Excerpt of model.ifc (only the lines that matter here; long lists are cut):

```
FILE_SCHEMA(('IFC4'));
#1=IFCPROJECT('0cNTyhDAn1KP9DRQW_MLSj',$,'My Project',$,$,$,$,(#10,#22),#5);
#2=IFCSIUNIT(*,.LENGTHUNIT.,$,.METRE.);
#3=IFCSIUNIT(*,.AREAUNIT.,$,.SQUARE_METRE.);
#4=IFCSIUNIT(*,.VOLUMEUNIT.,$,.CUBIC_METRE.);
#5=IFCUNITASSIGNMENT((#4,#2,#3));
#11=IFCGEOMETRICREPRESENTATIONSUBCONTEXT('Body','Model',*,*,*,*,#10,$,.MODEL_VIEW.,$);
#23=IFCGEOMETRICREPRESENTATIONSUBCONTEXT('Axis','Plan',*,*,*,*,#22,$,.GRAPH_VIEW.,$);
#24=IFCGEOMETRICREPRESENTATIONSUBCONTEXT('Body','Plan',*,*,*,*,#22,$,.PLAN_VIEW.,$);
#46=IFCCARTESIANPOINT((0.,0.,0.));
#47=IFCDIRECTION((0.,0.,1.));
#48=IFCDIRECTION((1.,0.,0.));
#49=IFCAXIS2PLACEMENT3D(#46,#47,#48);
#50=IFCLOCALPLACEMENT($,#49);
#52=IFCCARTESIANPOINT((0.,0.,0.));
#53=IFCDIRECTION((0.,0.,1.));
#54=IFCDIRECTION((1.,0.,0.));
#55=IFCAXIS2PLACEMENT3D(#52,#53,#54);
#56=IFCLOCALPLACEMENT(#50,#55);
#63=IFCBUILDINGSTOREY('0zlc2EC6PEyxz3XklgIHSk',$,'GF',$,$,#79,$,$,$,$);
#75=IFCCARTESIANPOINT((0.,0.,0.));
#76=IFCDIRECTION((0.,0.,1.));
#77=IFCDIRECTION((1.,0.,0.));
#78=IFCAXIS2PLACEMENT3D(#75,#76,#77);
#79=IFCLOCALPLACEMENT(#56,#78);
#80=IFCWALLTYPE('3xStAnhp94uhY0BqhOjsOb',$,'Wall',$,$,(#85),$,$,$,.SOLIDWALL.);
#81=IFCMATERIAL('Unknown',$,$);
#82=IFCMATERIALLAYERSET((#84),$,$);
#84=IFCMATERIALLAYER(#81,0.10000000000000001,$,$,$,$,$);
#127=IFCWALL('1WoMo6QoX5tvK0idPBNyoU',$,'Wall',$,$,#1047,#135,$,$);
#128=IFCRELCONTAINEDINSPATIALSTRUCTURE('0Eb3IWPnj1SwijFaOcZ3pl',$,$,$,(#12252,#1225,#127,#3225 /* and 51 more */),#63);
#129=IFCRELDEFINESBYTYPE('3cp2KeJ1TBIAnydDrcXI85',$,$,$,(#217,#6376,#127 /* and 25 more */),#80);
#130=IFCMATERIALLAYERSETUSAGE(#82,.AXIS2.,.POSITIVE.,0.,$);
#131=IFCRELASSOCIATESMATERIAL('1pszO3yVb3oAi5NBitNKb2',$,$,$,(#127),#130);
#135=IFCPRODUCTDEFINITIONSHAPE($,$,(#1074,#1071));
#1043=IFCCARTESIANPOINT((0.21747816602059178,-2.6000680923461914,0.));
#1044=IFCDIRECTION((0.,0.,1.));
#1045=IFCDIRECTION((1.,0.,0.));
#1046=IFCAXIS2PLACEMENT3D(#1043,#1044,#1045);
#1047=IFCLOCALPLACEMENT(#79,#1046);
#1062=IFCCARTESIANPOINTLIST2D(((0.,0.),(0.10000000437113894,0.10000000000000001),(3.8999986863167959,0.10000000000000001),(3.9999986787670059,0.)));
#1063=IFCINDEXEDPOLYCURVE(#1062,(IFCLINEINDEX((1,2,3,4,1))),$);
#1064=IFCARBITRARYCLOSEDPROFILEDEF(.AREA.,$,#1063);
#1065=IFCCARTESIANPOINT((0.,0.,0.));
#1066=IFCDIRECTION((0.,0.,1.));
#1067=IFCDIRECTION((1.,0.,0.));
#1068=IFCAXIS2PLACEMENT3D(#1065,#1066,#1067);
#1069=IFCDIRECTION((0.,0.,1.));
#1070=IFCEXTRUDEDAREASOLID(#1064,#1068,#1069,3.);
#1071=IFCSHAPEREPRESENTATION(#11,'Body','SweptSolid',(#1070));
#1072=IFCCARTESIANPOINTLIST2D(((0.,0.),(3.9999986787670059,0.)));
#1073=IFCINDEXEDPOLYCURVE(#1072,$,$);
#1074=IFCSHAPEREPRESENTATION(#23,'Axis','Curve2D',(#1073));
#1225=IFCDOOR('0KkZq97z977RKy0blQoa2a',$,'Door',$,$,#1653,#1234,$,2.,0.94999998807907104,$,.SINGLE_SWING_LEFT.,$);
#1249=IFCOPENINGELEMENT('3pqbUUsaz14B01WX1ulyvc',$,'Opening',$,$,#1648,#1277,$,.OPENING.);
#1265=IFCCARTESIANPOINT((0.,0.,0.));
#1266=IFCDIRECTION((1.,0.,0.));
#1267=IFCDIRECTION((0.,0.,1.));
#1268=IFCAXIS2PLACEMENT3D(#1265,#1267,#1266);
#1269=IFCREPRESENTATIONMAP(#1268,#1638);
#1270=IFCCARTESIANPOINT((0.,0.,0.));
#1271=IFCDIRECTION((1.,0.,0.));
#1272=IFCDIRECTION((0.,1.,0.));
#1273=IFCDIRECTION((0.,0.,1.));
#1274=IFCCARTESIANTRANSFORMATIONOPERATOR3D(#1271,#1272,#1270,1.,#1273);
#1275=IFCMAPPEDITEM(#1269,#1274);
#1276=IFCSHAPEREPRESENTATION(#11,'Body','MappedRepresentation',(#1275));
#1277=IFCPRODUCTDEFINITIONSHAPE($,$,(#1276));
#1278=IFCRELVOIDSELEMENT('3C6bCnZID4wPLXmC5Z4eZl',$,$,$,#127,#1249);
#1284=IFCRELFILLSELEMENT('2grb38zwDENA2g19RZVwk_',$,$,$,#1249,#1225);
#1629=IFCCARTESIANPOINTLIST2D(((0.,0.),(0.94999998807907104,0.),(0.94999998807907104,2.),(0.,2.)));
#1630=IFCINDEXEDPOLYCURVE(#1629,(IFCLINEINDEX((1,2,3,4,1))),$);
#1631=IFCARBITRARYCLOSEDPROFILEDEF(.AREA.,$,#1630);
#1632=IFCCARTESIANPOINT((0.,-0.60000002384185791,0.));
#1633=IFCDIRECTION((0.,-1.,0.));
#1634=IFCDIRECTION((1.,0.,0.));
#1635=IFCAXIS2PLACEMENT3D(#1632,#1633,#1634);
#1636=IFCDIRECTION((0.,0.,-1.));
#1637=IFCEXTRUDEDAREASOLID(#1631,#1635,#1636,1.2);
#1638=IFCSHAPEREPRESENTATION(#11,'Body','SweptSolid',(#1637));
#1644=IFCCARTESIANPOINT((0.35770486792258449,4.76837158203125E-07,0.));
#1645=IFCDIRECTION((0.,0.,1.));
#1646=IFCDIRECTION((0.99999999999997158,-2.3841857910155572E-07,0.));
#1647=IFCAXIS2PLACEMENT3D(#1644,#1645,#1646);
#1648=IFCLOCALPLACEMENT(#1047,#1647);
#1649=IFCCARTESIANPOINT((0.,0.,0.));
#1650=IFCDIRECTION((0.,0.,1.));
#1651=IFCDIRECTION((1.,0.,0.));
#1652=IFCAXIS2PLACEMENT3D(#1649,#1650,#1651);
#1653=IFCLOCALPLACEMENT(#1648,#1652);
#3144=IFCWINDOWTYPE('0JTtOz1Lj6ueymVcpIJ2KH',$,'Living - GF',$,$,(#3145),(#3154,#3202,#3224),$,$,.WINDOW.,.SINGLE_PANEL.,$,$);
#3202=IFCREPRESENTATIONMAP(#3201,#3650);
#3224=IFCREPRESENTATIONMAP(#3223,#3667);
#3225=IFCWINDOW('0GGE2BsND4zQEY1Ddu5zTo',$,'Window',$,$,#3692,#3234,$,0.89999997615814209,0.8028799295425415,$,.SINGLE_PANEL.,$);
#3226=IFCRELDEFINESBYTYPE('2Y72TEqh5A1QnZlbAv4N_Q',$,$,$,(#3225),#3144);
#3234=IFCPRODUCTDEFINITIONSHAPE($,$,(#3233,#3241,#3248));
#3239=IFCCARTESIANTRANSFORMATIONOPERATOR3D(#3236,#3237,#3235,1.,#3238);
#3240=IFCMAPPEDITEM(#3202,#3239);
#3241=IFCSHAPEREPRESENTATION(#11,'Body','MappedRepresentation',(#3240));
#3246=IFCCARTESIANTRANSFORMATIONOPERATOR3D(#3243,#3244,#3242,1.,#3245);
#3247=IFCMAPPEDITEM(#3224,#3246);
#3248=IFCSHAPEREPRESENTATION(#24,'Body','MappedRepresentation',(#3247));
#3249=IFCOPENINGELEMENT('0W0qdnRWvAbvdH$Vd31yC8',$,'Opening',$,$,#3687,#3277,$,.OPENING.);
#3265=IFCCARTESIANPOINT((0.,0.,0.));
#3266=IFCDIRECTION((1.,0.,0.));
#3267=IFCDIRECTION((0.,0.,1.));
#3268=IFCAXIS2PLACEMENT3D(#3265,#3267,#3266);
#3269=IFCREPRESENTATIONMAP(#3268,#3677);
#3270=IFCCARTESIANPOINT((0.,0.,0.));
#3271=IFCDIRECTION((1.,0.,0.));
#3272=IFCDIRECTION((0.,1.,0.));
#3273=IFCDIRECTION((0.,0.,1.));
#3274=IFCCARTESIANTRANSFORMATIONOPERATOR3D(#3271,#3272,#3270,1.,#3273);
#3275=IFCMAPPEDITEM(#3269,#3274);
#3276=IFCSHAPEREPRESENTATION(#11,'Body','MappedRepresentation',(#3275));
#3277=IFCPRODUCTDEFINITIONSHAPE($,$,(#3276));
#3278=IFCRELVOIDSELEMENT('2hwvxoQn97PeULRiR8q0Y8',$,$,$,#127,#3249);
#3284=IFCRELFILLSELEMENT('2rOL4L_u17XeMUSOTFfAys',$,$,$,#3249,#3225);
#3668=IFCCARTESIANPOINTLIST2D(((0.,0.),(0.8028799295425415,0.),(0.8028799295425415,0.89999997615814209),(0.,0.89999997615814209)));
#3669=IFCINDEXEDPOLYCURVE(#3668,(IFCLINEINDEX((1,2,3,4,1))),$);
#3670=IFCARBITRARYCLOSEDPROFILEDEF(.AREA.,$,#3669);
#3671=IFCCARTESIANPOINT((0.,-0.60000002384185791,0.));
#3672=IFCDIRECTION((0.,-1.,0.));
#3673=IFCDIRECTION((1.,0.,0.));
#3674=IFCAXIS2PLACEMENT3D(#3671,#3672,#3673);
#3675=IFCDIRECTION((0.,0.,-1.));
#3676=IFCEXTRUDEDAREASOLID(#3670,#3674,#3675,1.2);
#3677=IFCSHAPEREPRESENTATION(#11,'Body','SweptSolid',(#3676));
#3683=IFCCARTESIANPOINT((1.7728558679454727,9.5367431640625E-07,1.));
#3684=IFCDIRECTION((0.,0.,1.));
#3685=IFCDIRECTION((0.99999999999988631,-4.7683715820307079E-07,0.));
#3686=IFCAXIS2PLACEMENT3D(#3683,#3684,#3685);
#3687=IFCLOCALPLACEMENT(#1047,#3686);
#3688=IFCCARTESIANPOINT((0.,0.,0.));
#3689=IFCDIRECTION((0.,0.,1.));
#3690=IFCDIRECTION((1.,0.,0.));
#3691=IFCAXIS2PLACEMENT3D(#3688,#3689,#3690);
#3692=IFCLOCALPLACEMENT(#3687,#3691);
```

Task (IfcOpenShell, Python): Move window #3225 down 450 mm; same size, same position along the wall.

```python
import numpy as np
import ifcopenshell
import ifcopenshell.api.geometry
import ifcopenshell.util.placement
import ifcopenshell.util.unit

model = ifcopenshell.open("model.ifc")
unit_scale = ifcopenshell.util.unit.calculate_unit_scale(model)

window = model.by_guid("0GGE2BsND4zQEY1Ddu5zTo")
opening = window.FillsVoids[0].RelatingOpeningElement
dz = -0.45

shift = np.array([0.0, 0.0, dz])
# The window is placed relative to its opening, so it follows when the opening moves.
matrix = ifcopenshell.util.placement.get_local_placement(opening.ObjectPlacement)
matrix[:3, 3] += shift
ifcopenshell.api.geometry.edit_object_placement(
    model, product=opening, matrix=matrix, is_si=False, should_transform_children=True
)

print(f"moved by {dz * unit_scale:+.3f} m")

model.write("model_updated.ifc")
```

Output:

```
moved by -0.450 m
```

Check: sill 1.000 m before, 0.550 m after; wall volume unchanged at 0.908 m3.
